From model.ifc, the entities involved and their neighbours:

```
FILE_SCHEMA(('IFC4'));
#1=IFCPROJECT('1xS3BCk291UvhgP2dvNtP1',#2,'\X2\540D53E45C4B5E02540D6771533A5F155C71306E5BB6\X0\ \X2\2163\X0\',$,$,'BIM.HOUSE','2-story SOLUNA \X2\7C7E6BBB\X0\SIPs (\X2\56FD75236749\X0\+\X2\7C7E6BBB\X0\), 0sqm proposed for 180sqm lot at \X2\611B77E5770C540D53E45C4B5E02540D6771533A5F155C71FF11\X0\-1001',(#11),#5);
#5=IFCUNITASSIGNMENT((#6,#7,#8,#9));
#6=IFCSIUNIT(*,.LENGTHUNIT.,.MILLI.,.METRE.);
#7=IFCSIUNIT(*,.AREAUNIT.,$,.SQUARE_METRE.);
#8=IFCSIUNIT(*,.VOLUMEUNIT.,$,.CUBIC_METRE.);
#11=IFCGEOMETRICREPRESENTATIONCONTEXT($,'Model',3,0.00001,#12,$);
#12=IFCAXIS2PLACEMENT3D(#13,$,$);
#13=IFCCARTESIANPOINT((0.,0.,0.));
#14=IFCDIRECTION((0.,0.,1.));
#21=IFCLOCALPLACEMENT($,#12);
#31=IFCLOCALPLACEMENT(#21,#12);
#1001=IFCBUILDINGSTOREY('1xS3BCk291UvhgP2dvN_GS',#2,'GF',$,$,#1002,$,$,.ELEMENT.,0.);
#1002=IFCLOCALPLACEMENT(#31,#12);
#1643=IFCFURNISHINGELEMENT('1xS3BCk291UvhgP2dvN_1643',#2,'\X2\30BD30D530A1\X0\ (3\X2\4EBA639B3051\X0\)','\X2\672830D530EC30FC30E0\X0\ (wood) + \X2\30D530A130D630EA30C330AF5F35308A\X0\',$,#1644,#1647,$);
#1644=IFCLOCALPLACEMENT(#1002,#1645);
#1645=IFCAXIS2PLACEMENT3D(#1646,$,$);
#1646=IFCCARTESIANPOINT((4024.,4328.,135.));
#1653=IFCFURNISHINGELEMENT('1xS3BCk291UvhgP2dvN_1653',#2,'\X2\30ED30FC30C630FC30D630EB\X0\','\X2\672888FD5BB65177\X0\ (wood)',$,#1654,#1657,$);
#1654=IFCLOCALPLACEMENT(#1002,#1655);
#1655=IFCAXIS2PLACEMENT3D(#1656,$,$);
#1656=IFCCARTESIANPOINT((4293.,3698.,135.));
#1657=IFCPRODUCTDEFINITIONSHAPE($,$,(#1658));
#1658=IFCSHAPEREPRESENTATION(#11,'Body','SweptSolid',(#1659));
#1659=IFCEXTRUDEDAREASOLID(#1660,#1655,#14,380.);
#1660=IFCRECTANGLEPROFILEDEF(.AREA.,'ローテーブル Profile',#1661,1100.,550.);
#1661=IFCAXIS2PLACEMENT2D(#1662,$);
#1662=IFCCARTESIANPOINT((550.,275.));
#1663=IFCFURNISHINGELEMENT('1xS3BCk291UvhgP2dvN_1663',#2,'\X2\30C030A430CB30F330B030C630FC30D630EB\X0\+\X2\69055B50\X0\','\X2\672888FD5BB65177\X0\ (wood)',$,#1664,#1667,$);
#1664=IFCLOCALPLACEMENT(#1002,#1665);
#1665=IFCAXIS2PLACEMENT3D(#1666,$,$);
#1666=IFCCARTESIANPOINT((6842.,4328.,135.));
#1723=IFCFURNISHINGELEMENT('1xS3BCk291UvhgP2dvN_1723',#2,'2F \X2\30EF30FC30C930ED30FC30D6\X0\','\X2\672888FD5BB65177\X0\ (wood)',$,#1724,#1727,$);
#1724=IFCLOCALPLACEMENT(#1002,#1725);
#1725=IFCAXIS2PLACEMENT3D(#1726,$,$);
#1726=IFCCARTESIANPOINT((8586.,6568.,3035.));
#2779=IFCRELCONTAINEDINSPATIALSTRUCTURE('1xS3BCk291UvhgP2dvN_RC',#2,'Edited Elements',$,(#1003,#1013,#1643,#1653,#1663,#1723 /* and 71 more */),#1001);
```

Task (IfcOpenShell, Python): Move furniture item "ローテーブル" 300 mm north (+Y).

```python
import ifcopenshell
import ifcopenshell.api.geometry
import ifcopenshell.util.placement

model = ifcopenshell.open("model.ifc")

item = model.by_guid("1xS3BCk291UvhgP2dvN_1653")
matrix = ifcopenshell.util.placement.get_local_placement(item.ObjectPlacement)
matrix[1, 3] += 300.0
ifcopenshell.api.geometry.edit_object_placement(model, product=item, matrix=matrix, is_si=False)

print(ifcopenshell.util.placement.get_local_placement(item.ObjectPlacement).round(3) + 0.0)

model.write("model-out.ifc")
```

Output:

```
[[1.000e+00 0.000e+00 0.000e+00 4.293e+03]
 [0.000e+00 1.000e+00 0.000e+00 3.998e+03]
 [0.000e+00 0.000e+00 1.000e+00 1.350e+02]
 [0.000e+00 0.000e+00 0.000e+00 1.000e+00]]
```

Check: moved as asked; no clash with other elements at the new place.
